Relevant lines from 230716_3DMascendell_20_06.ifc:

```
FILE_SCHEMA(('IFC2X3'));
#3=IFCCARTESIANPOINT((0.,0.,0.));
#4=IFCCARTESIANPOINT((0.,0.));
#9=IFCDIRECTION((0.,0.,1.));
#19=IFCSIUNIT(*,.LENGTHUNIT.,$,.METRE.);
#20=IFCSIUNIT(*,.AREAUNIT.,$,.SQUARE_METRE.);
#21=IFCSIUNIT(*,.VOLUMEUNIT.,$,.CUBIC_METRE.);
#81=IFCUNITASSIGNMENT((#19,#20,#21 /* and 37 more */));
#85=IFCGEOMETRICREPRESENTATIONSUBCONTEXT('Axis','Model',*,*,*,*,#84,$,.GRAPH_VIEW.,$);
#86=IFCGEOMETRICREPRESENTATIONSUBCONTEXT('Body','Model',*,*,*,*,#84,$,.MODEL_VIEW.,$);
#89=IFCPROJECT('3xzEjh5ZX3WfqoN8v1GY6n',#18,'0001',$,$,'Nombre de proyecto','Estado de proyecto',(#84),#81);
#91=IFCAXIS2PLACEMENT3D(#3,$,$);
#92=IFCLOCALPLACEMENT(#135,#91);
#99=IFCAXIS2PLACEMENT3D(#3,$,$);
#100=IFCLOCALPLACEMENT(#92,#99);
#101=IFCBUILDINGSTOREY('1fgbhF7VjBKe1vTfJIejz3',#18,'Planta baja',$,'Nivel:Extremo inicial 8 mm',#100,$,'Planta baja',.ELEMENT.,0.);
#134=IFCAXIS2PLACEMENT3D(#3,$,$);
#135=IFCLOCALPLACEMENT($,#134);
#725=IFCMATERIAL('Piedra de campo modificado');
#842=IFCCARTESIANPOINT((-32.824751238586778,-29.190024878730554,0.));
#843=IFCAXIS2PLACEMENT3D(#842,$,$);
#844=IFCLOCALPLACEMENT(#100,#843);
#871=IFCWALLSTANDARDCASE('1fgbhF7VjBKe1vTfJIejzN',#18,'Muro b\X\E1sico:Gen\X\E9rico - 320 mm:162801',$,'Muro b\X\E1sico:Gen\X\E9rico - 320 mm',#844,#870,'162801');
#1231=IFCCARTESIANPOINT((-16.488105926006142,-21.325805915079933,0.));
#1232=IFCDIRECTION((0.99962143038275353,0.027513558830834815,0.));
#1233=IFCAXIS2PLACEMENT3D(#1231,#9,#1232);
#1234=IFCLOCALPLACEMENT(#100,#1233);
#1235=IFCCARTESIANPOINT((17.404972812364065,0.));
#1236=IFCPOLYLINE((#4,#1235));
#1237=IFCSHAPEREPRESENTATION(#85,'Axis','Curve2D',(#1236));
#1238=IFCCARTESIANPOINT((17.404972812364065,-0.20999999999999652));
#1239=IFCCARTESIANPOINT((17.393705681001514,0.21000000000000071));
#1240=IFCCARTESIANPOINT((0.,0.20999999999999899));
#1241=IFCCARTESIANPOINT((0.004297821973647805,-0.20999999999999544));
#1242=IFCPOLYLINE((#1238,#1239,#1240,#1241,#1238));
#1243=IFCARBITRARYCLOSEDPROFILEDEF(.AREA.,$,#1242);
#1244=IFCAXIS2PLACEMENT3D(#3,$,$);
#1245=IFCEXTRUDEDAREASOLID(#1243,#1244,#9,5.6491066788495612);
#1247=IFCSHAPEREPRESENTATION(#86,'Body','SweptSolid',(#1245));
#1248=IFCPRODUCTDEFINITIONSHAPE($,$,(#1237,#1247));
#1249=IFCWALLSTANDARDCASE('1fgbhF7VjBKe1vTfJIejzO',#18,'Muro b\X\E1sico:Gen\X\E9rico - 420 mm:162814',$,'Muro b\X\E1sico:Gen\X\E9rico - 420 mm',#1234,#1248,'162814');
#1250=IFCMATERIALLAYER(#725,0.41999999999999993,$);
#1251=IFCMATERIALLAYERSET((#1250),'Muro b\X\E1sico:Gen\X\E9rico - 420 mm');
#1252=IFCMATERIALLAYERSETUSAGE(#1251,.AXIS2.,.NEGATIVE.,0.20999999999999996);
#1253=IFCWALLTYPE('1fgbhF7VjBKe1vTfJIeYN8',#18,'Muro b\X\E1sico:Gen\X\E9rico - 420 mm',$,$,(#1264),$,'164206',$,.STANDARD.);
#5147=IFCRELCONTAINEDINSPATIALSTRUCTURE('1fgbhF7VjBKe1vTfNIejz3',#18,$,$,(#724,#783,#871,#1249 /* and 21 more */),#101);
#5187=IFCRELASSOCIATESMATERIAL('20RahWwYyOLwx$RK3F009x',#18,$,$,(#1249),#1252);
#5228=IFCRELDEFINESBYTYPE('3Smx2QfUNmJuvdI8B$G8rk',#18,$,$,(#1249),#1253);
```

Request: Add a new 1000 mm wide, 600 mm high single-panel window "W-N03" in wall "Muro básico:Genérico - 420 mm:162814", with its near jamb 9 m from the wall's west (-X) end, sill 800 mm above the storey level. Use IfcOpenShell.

```python
import numpy as np
import ifcopenshell
import ifcopenshell.api.feature
import ifcopenshell.api.geometry
import ifcopenshell.api.root
import ifcopenshell.api.spatial
import ifcopenshell.api.type
import ifcopenshell.geom
import ifcopenshell.util.element
import ifcopenshell.util.placement
import ifcopenshell.util.representation
import ifcopenshell.util.shape
import ifcopenshell.util.unit

model = ifcopenshell.open("230716_3DMascendell_20_06.ifc")
unit_scale = ifcopenshell.util.unit.calculate_unit_scale(model)
settings = ifcopenshell.geom.settings()


def volume(element):
    """Net volume in cubic metres, openings subtracted."""
    shape = ifcopenshell.geom.create_shape(settings, element)
    return ifcopenshell.util.shape.get_volume(shape.geometry)


wall = model.by_guid("1fgbhF7VjBKe1vTfJIejzO")
storey = ifcopenshell.util.element.get_container(wall, ifc_class="IfcBuildingStorey")
context = ifcopenshell.util.representation.get_context(model, "Model", "Body", "MODEL_VIEW")
before = volume(wall)

width, height, from_end, sill = 1, 0.6, 9, 0.8  # metres

# The wall runs along its own X axis, and the end named is its -X end.
wall_shape = ifcopenshell.geom.create_shape(settings, wall)
x, y, z = ifcopenshell.util.shape.get_vertices(wall_shape.geometry).T
start = x.min() + from_end
face, thickness = float(y.min()), float(y.max() - y.min())
wall_matrix = ifcopenshell.util.placement.get_local_placement(wall.ObjectPlacement)
level = ifcopenshell.util.placement.get_local_placement(storey.ObjectPlacement)[2, 3]


def in_wall(x, y):
    """Placement at x, y metres in the wall's axes, at sill height."""
    matrix = wall_matrix.copy()
    matrix[:, 3] = wall_matrix @ np.array([x / unit_scale, y / unit_scale, 0.0, 1.0])
    matrix[2, 3] = level + sill / unit_scale
    return matrix


# Opening: a box that overshoots both wall faces by 50 mm.
opening = ifcopenshell.api.root.create_entity(model, ifc_class="IfcOpeningElement")
box = ifcopenshell.api.geometry.add_wall_representation(
    model, context=context, length=width, height=height, thickness=thickness + 0.1
)
ifcopenshell.api.geometry.assign_representation(model, product=opening, representation=box)
ifcopenshell.api.geometry.edit_object_placement(model, product=opening, matrix=in_wall(start, face - 0.05), is_si=False)
ifcopenshell.api.feature.add_feature(model, feature=opening, element=wall)

window = ifcopenshell.api.root.create_entity(model, ifc_class="IfcWindow", name="W-N03")
window.OverallWidth, window.OverallHeight = width / unit_scale, height / unit_scale
body = ifcopenshell.api.geometry.add_window_representation(
    model,
    context=context,
    overall_width=window.OverallWidth,
    overall_height=window.OverallHeight,
    partition_type="SINGLE_PANEL",
)
ifcopenshell.api.geometry.assign_representation(model, product=window, representation=body)
ifcopenshell.api.spatial.assign_container(model, products=[window], relating_structure=storey)
fills = ifcopenshell.api.feature.add_filling(model, opening=opening, element=window)
fills.OwnerHistory = window.OwnerHistory  # required in IFC2X3

# IFC2X3 keeps the operation on the window style.
style = ifcopenshell.api.root.create_entity(model, ifc_class="IfcWindowStyle", name="W-N03")
style.OperationType, style.ConstructionType = "SINGLE_PANEL", "NOTDEFINED"
style.ParameterTakesPrecedence = style.Sizeable = False
ifcopenshell.api.type.assign_type(model, related_objects=[window], relating_type=style)

# Centre the window in the wall's thickness.
ifcopenshell.api.geometry.edit_object_placement(model, product=window, matrix=in_wall(start, face), is_si=False)
window_shape = ifcopenshell.geom.create_shape(settings, window)
depth = ifcopenshell.util.shape.get_vertices(window_shape.geometry)[:, 1]
offset = face + thickness / 2 - (depth.min() + depth.max()) / 2
ifcopenshell.api.geometry.edit_object_placement(model, product=window, matrix=in_wall(start, offset), is_si=False)

after = volume(wall)

print(f"wall volume {before:.3f} -> {after:.3f} m3")

model.write("230716_3DMascendell_20_06_v2.ifc")
```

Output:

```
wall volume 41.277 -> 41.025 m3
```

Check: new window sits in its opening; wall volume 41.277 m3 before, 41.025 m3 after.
